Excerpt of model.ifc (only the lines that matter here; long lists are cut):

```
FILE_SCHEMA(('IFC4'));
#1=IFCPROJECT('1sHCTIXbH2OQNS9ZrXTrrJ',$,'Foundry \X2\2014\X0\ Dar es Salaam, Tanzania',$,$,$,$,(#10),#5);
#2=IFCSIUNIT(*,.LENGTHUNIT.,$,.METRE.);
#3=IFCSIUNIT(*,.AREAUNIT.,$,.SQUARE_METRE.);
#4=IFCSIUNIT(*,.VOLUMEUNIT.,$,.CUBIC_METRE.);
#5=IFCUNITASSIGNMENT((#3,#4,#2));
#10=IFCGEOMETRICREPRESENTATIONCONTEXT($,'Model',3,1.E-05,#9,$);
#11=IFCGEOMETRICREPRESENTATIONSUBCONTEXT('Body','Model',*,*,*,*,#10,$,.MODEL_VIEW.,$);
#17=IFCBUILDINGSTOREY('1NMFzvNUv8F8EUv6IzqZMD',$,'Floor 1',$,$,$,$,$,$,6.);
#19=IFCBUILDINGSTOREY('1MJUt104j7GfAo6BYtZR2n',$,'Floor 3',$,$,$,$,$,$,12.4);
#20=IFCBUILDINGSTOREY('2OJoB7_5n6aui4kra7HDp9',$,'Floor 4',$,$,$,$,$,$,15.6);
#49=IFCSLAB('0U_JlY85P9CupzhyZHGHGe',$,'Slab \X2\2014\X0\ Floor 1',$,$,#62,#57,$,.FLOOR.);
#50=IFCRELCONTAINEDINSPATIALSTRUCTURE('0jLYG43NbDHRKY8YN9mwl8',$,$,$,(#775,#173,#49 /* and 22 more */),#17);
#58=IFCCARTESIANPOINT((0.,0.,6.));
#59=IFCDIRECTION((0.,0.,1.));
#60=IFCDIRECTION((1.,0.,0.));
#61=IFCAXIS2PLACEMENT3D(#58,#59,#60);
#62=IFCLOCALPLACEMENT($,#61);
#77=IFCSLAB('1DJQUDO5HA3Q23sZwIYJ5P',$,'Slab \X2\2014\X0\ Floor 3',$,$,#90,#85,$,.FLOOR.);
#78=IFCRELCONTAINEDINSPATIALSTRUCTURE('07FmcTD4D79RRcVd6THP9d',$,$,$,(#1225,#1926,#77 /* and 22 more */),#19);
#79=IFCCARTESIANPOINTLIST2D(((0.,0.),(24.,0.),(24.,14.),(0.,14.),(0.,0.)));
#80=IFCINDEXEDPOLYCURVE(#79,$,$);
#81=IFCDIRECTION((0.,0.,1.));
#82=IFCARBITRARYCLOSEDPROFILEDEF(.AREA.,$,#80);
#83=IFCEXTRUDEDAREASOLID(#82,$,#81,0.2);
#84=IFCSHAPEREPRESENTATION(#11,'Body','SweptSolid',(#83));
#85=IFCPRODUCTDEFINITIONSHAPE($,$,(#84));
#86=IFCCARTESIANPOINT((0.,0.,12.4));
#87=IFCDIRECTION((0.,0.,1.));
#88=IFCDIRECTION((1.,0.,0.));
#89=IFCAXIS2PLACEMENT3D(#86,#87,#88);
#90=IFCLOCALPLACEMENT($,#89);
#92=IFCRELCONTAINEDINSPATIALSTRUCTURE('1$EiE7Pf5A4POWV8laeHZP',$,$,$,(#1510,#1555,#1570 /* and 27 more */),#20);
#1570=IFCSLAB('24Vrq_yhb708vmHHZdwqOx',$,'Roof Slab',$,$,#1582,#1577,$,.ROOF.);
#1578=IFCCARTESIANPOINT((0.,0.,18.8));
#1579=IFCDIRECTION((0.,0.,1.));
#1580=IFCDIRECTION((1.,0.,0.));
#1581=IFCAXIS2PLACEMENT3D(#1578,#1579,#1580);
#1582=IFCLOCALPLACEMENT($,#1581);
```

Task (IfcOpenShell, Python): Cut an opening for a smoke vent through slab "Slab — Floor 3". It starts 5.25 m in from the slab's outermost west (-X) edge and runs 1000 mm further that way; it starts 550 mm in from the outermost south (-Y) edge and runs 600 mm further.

```python
import numpy as np
import ifcopenshell
import ifcopenshell.api.feature
import ifcopenshell.api.geometry
import ifcopenshell.api.root
import ifcopenshell.geom
import ifcopenshell.util.placement
import ifcopenshell.util.representation
import ifcopenshell.util.shape
import ifcopenshell.util.unit

model = ifcopenshell.open("model.ifc")
unit_scale = ifcopenshell.util.unit.calculate_unit_scale(model)
settings = ifcopenshell.geom.settings()


def volume(element):
    """Net volume in cubic metres, openings subtracted."""
    shape = ifcopenshell.geom.create_shape(settings, element)
    return ifcopenshell.util.shape.get_volume(shape.geometry)


slab = model.by_id(77)
before = volume(slab)

# Extent in the slab's own axes, in metres. The edges named are its -X and -Y sides.
slab_shape = ifcopenshell.geom.create_shape(settings, slab)
vertices = ifcopenshell.util.shape.get_vertices(slab_shape.geometry)
x_min, y_min, bottom = vertices.min(axis=0)
top = vertices[:, 2].max()

opening = ifcopenshell.api.root.create_entity(model, ifc_class="IfcOpeningElement", name="Smoke vent opening", predefined_type="OPENING")
context = ifcopenshell.util.representation.get_context(model, "Model", "Body", "MODEL_VIEW")
width, depth = 1, 0.6
outline = [(0.0, 0.0), (width, 0.0), (width, depth), (0.0, depth), (0.0, 0.0)]
# Overshoot both faces by 50 mm so the cut is clean.
shape = ifcopenshell.api.geometry.add_slab_representation(
    model, context=context, depth=top - bottom + 0.1, polyline=outline
)
ifcopenshell.api.geometry.assign_representation(model, product=opening, representation=shape)

matrix = ifcopenshell.util.placement.get_local_placement(slab.ObjectPlacement)
matrix[:, 3] = matrix @ np.append(np.array([x_min + 5.25, y_min + 0.55, bottom - 0.05]) / unit_scale, 1.0)
ifcopenshell.api.geometry.edit_object_placement(model, product=opening, matrix=matrix, is_si=False)
ifcopenshell.api.feature.add_feature(model, feature=opening, element=slab)

after = volume(slab)

print(f"slab volume {before:.3f} -> {after:.3f} m3")

model.write("model-out.ifc")
```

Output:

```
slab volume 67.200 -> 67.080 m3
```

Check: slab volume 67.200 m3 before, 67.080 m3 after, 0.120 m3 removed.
